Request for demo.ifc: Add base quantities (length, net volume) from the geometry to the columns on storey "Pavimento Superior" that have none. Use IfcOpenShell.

First a look at what the model holds.

```python
import ifcopenshell
import ifcopenshell.util.element
import ifcopenshell.util.unit

model = ifcopenshell.open("demo.ifc")
print(model.schema)
for unit_type in ("LENGTHUNIT", "AREAUNIT", "VOLUMEUNIT"):
    print(unit_type, ifcopenshell.util.unit.calculate_unit_scale(model, unit_type))
storey = next(s for s in model.by_type("IfcBuildingStorey") if s.Name == "Pavimento Superior")
columns = [e for e in ifcopenshell.util.element.get_decomposition(storey) if e.is_a("IfcColumn")]
for e in sorted(columns, key=lambda e: e.id()):
    print(e.id(), e.is_a(), e.Name, list(ifcopenshell.util.element.get_psets(e, qtos_only=True)), sep=" | ")
```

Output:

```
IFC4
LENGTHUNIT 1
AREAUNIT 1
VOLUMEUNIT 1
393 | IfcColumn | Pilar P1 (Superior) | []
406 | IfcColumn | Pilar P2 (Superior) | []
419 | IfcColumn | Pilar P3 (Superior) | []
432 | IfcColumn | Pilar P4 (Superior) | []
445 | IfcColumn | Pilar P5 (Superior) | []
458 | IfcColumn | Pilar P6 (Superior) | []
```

```python
import ifcopenshell
import ifcopenshell.api.pset
import ifcopenshell.geom
import ifcopenshell.util.element
import ifcopenshell.util.shape
import ifcopenshell.util.unit

model = ifcopenshell.open("demo.ifc")
unit_scale = ifcopenshell.util.unit.calculate_unit_scale(model)
volume_scale = ifcopenshell.util.unit.calculate_unit_scale(model, "VOLUMEUNIT")
settings = ifcopenshell.geom.settings()

storey = next(s for s in model.by_type("IfcBuildingStorey") if s.Name == "Pavimento Superior")
columns = [e for e in ifcopenshell.util.element.get_decomposition(storey) if e.is_a("IfcColumn")]

for e in sorted(columns, key=lambda e: e.id()):
    if ifcopenshell.util.element.get_psets(e, qtos_only=True, should_inherit=False):
        continue
    # Geometry comes back in metres, in the element's own axes.
    shape = ifcopenshell.geom.create_shape(settings, e)
    values = {
        "Length": ifcopenshell.util.shape.get_z(shape.geometry) / unit_scale,
        "NetVolume": ifcopenshell.util.shape.get_volume(shape.geometry) / volume_scale,
    }
    qto = ifcopenshell.api.pset.add_qto(model, product=e, name="Qto_ColumnBaseQuantities")
    ifcopenshell.api.pset.edit_qto(model, qto=qto, properties=values)
    print(e.id(), {k: round(v, 3) for k, v in values.items()})

model.write("demo_rev.ifc")
```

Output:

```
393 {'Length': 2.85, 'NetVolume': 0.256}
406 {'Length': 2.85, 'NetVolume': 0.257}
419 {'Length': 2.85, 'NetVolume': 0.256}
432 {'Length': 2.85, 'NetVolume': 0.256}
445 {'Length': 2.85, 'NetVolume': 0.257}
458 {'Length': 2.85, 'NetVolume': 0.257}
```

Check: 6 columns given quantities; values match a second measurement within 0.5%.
